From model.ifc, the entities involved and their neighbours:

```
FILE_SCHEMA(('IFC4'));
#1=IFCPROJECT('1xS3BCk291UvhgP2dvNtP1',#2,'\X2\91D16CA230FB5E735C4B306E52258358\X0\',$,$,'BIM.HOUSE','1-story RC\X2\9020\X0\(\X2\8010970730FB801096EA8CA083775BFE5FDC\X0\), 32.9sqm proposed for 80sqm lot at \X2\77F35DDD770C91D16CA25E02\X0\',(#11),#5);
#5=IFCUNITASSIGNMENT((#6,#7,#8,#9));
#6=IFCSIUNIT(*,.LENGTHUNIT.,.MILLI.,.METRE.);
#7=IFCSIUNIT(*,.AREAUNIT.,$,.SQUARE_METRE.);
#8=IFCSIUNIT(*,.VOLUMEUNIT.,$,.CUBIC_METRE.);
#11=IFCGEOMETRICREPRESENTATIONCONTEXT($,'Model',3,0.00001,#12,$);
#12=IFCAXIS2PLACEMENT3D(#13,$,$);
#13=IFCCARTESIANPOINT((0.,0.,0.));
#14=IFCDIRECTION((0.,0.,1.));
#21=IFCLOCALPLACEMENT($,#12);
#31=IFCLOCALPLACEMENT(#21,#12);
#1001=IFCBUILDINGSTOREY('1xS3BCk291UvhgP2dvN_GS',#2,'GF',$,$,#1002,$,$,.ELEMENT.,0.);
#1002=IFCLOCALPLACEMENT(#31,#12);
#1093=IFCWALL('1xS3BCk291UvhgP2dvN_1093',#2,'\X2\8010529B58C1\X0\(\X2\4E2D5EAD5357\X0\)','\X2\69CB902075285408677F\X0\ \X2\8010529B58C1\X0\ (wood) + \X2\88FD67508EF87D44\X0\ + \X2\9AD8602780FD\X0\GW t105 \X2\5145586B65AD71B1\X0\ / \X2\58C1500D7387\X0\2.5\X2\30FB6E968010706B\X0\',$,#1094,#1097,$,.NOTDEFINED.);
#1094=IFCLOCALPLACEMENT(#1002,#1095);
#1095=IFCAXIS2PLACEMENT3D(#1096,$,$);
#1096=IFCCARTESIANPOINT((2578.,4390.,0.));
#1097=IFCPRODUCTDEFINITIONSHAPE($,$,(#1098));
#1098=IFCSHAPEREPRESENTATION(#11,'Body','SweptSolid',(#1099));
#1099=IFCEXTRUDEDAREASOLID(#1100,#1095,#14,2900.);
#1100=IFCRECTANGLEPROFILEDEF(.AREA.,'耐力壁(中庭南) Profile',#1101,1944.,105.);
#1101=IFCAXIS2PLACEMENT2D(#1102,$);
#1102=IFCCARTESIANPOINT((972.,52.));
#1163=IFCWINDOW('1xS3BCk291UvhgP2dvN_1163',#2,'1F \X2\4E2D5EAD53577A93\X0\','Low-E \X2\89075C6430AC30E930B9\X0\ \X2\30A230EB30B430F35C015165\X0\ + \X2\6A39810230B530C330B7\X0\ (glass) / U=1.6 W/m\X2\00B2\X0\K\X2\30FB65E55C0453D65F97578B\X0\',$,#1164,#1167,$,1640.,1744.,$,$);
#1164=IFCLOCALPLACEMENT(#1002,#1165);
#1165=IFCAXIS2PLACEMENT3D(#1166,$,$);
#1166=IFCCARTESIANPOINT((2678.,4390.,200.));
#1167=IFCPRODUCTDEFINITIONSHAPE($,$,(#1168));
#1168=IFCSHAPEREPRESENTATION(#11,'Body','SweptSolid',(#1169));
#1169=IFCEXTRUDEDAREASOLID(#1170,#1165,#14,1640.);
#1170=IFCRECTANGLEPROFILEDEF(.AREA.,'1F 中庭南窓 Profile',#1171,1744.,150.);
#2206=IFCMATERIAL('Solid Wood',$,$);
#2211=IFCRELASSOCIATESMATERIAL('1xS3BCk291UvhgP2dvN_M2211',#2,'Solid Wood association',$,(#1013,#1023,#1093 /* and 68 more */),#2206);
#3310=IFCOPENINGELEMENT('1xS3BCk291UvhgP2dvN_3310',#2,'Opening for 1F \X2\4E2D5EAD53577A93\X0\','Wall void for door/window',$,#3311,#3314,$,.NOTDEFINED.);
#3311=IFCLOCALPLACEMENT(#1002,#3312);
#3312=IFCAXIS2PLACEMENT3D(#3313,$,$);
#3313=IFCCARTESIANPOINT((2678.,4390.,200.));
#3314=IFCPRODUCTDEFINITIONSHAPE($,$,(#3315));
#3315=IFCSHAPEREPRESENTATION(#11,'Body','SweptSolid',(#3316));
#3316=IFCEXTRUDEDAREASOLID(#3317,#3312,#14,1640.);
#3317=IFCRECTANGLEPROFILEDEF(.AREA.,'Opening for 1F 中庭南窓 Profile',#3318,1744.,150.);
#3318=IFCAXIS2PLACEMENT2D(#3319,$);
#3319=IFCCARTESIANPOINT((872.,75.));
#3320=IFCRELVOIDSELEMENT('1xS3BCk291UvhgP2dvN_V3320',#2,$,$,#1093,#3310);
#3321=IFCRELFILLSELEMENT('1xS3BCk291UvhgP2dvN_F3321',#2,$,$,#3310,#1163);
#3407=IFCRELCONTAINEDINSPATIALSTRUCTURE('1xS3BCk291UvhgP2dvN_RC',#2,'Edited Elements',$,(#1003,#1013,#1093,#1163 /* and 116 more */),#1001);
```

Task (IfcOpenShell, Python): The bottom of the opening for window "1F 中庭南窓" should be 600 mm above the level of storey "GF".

```python
import numpy as np
import ifcopenshell
import ifcopenshell.api.geometry
import ifcopenshell.geom
import ifcopenshell.util.element
import ifcopenshell.util.placement
import ifcopenshell.util.shape
import ifcopenshell.util.unit

model = ifcopenshell.open("model.ifc")
unit_scale = ifcopenshell.util.unit.calculate_unit_scale(model)

window = model.by_guid("1xS3BCk291UvhgP2dvN_1163")
opening = window.FillsVoids[0].RelatingOpeningElement
storey = ifcopenshell.util.element.get_container(window, ifc_class="IfcBuildingStorey")
level = ifcopenshell.util.placement.get_local_placement(storey.ObjectPlacement)[2, 3]

# The opening's origin need not be at the sill, so measure its lowest point.
shape = ifcopenshell.geom.create_shape(ifcopenshell.geom.settings(), opening)
bottom = ifcopenshell.util.shape.get_shape_bottom_elevation(shape, shape.geometry) / unit_scale
dz = level + 0.6 / unit_scale - bottom

shift = np.array([0.0, 0.0, dz])
# The window is not placed relative to its opening, so move both.
for product in (opening, window):
    matrix = ifcopenshell.util.placement.get_local_placement(product.ObjectPlacement)
    matrix[:3, 3] += shift
    ifcopenshell.api.geometry.edit_object_placement(model, product=product, matrix=matrix, is_si=False)

print(f"moved by {dz * unit_scale:+.3f} m")

model.write("model_rev.ifc")
```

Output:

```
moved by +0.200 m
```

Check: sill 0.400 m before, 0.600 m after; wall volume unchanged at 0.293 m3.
